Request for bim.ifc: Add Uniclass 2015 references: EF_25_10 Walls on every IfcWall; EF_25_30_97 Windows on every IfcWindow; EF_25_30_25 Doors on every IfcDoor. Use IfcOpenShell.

First a look at what the model holds.

```python
import ifcopenshell

model = ifcopenshell.open("bim.ifc")
print(model.schema)
print("classifications:", [c.Name for c in model.by_type("IfcClassification")])
for ifc_class in ("IfcDoor", "IfcRoof", "IfcStair", "IfcWall", "IfcWindow"):
    print(ifc_class, len(model.by_type(ifc_class)))
```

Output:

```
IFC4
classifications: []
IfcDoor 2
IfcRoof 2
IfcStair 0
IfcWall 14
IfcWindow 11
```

```python
import ifcopenshell
import ifcopenshell.api.classification

model = ifcopenshell.open("bim.ifc")

system = ifcopenshell.api.classification.add_classification(model, classification="Uniclass 2015")

codes = {
    "IfcWall": ("EF_25_10", "Walls"),
    "IfcWindow": ("EF_25_30_97", "Windows"),
    "IfcDoor": ("EF_25_30_25", "Doors"),
}
for ifc_class, (code, name) in codes.items():
    products = model.by_type(ifc_class)
    ifcopenshell.api.classification.add_reference(
        model, products=products, classification=system, identification=code, name=name
    )
    print(code, len(products))

model.write("bim_rev.ifc")
```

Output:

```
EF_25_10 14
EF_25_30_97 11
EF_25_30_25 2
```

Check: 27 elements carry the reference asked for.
